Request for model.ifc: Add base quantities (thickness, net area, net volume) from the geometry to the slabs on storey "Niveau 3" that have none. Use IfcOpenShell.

First a look at what the model holds.

```python
import ifcopenshell
import ifcopenshell.util.element
import ifcopenshell.util.unit

model = ifcopenshell.open("model.ifc")
print(model.schema)
for unit_type in ("LENGTHUNIT", "AREAUNIT", "VOLUMEUNIT"):
    print(unit_type, ifcopenshell.util.unit.calculate_unit_scale(model, unit_type))
storey = next(s for s in model.by_type("IfcBuildingStorey") if s.Name == "Niveau 3")
slabs = [e for e in ifcopenshell.util.element.get_decomposition(storey) if e.is_a("IfcSlab")]
for e in sorted(slabs, key=lambda e: e.id()):
    print(e.id(), e.is_a(), e.Name, list(ifcopenshell.util.element.get_psets(e, qtos_only=True)), sep=" | ")
```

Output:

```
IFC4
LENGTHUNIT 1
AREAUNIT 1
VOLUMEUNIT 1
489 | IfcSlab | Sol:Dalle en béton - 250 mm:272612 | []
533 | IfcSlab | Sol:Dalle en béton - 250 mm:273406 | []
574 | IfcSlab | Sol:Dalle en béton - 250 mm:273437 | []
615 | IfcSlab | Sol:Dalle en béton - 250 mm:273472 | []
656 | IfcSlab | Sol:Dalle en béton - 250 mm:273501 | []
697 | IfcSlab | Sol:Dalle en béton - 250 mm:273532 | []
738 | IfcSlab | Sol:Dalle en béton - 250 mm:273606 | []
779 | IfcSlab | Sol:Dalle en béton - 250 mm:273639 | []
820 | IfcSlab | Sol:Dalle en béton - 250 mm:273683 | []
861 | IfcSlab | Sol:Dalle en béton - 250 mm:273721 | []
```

```python
import ifcopenshell
import ifcopenshell.api.pset
import ifcopenshell.geom
import ifcopenshell.util.element
import ifcopenshell.util.shape
import ifcopenshell.util.unit

model = ifcopenshell.open("model.ifc")
unit_scale = ifcopenshell.util.unit.calculate_unit_scale(model)
area_scale = ifcopenshell.util.unit.calculate_unit_scale(model, "AREAUNIT")
volume_scale = ifcopenshell.util.unit.calculate_unit_scale(model, "VOLUMEUNIT")
settings = ifcopenshell.geom.settings()

storey = next(s for s in model.by_type("IfcBuildingStorey") if s.Name == "Niveau 3")
slabs = [e for e in ifcopenshell.util.element.get_decomposition(storey) if e.is_a("IfcSlab")]

for e in sorted(slabs, key=lambda e: e.id()):
    if ifcopenshell.util.element.get_psets(e, qtos_only=True, should_inherit=False):
        continue
    # Geometry comes back in metres, in the element's own axes.
    shape = ifcopenshell.geom.create_shape(settings, e)
    values = {
        "Width": ifcopenshell.util.shape.get_z(shape.geometry) / unit_scale,
        "NetArea": ifcopenshell.util.shape.get_footprint_area(shape.geometry) / area_scale,
        "NetVolume": ifcopenshell.util.shape.get_volume(shape.geometry) / volume_scale,
    }
    qto = ifcopenshell.api.pset.add_qto(model, product=e, name="Qto_SlabBaseQuantities")
    ifcopenshell.api.pset.edit_qto(model, qto=qto, properties=values)
    print(e.id(), {k: round(v, 3) for k, v in values.items()})

model.write("model_v2.ifc")
```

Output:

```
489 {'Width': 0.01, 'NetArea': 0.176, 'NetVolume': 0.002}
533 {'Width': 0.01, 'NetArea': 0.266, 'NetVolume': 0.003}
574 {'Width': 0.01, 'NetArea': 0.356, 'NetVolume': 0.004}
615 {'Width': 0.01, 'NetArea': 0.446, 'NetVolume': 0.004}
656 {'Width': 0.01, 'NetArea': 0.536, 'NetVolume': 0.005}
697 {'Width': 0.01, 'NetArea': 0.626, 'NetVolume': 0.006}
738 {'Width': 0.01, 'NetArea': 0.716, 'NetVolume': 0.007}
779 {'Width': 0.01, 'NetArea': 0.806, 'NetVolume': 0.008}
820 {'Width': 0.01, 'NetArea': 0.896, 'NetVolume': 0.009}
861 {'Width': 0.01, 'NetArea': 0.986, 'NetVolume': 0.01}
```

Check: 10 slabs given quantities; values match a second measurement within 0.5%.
